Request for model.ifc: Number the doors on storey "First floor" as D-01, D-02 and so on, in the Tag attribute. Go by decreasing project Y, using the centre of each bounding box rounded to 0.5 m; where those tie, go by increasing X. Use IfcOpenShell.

First a look at what the model holds.

```python
import ifcopenshell
import ifcopenshell.util.element
import ifcopenshell.util.placement

model = ifcopenshell.open("model.ifc")
print(model.schema)
storey = next(s for s in model.by_type("IfcBuildingStorey") if s.Name == "First floor")
doors = [e for e in ifcopenshell.util.element.get_decomposition(storey) if e.is_a("IfcDoor")]
for e in sorted(doors, key=lambda e: e.id()):
    origin = ifcopenshell.util.placement.get_local_placement(e.ObjectPlacement)[:3, 3]
    print(e.id(), e.Tag, e.Name, origin.round(2) + 0.0, sep=" | ")
```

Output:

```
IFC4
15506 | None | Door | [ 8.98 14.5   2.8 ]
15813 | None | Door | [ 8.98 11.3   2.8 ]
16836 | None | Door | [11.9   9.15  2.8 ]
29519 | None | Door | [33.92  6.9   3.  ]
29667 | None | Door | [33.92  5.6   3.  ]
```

```python
import ifcopenshell
import ifcopenshell.geom
import ifcopenshell.util.element
import ifcopenshell.util.shape

model = ifcopenshell.open("model.ifc")
settings = ifcopenshell.geom.settings()
settings.set("use-world-coords", True)


def centre(element):
    shape = ifcopenshell.geom.create_shape(settings, element)
    return ifcopenshell.util.shape.get_bbox_centroid(shape.geometry)


storey = next(s for s in model.by_type("IfcBuildingStorey") if s.Name == "First floor")
doors = [e for e in ifcopenshell.util.element.get_decomposition(storey) if e.is_a("IfcDoor")]

# Insertion points can sit at a corner or the storey origin, so sort by the geometry (in metres).
centres = {e: centre(e) for e in doors}
doors.sort(key=lambda e: (-round(centres[e][1] / 0.5), centres[e][0]))

for i, e in enumerate(doors, start=1):
    number = f"D-{i:02d}"
    e.Tag = number
    print(e.id(), number)

model.write("model_updated.ifc")
```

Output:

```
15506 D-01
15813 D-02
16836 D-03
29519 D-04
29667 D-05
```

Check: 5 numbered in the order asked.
